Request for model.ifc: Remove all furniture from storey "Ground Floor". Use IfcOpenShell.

First a look at what the model holds.

```python
import ifcopenshell
import ifcopenshell.util.element

model = ifcopenshell.open("model.ifc")
print(model.schema)
storey = next(s for s in model.by_type("IfcBuildingStorey") if s.Name == "Ground Floor")
furniture = [e for e in ifcopenshell.util.element.get_decomposition(storey) if e.is_a("IfcFurnishingElement")]
seen = {}
for e in furniture:
    element_type = ifcopenshell.util.element.get_type(e)
    name = element_type.Name if element_type not in (None, e) else None
    seen[name] = seen.get(name, 0) + 1
for name, count in sorted(seen.items(), key=str):
    print(count, "x", name)
```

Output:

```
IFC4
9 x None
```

```python
import ifcopenshell
import ifcopenshell.api.root
import ifcopenshell.util.element

model = ifcopenshell.open("model.ifc")

storey = next(s for s in model.by_type("IfcBuildingStorey") if s.Name == "Ground Floor")
furniture = [e for e in ifcopenshell.util.element.get_decomposition(storey) if e.is_a("IfcFurnishingElement")]

for e in furniture:
    ifcopenshell.api.root.remove_product(model, product=e)
print(len(furniture), "removed")

model.write("model_updated.ifc")
```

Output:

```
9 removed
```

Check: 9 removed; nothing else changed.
